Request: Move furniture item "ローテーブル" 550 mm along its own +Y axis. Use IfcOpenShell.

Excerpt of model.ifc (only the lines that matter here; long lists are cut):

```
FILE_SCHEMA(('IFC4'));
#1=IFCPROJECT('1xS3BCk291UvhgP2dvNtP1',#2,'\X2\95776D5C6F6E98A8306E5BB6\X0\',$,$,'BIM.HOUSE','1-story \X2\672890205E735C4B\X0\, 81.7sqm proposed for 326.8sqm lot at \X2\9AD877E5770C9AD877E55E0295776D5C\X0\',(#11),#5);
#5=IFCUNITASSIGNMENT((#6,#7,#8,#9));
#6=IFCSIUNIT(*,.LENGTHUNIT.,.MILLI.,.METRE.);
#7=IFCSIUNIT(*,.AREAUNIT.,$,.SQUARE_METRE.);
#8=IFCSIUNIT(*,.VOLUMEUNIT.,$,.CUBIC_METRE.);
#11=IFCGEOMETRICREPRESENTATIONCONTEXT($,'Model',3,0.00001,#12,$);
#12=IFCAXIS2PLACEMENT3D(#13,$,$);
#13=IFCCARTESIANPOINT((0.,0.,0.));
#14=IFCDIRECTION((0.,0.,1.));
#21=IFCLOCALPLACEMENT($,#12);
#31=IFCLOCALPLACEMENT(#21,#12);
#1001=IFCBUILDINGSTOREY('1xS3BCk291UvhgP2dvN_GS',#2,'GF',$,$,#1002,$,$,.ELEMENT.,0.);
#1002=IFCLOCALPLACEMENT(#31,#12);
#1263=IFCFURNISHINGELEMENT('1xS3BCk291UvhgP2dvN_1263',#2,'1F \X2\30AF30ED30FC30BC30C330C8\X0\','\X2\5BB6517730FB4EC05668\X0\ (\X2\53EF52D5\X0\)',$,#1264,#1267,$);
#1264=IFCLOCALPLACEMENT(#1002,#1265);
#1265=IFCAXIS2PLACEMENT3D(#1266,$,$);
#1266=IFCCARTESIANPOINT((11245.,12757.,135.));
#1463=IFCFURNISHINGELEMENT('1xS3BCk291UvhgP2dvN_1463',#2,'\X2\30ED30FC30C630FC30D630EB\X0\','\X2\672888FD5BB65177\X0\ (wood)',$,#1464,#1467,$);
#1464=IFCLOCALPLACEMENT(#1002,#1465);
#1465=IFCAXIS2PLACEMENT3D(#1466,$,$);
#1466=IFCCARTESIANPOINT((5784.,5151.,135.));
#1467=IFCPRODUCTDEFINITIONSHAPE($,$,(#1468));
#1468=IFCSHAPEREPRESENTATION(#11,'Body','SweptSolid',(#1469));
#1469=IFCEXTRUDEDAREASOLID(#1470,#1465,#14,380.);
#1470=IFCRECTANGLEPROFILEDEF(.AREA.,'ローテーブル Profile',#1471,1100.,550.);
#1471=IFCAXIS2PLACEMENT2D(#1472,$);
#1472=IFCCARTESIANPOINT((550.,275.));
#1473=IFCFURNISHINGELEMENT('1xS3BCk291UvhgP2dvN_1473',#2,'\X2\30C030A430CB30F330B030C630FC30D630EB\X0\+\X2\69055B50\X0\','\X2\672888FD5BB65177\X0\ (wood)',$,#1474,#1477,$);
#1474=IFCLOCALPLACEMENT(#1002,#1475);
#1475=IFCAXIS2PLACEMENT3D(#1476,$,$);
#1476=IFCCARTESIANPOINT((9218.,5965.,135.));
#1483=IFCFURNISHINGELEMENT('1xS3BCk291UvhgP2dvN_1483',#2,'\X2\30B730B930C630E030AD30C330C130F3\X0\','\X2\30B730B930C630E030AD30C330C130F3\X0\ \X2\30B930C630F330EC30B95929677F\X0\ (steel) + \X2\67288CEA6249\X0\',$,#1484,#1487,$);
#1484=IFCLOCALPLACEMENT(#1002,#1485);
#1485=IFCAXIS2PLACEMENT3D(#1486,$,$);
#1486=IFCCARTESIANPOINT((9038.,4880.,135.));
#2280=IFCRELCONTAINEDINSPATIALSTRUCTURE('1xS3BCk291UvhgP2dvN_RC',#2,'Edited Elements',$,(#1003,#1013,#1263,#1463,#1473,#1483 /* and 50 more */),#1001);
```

```python
import ifcopenshell
import ifcopenshell.api.geometry
import ifcopenshell.util.placement
import ifcopenshell.util.unit

model = ifcopenshell.open("model.ifc")
unit_scale = ifcopenshell.util.unit.calculate_unit_scale(model)

item = model.by_guid("1xS3BCk291UvhgP2dvN_1463")
matrix = ifcopenshell.util.placement.get_local_placement(item.ObjectPlacement)
matrix[:3, 3] += matrix[:3, 1] * 0.55 / unit_scale
ifcopenshell.api.geometry.edit_object_placement(model, product=item, matrix=matrix, is_si=False)

print(ifcopenshell.util.placement.get_local_placement(item.ObjectPlacement).round(3) + 0.0)

model.write("model_edited.ifc")
```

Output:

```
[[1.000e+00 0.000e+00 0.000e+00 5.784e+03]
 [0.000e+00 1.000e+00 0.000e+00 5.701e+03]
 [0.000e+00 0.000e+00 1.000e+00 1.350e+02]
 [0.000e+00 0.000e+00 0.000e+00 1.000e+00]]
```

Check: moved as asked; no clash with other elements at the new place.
